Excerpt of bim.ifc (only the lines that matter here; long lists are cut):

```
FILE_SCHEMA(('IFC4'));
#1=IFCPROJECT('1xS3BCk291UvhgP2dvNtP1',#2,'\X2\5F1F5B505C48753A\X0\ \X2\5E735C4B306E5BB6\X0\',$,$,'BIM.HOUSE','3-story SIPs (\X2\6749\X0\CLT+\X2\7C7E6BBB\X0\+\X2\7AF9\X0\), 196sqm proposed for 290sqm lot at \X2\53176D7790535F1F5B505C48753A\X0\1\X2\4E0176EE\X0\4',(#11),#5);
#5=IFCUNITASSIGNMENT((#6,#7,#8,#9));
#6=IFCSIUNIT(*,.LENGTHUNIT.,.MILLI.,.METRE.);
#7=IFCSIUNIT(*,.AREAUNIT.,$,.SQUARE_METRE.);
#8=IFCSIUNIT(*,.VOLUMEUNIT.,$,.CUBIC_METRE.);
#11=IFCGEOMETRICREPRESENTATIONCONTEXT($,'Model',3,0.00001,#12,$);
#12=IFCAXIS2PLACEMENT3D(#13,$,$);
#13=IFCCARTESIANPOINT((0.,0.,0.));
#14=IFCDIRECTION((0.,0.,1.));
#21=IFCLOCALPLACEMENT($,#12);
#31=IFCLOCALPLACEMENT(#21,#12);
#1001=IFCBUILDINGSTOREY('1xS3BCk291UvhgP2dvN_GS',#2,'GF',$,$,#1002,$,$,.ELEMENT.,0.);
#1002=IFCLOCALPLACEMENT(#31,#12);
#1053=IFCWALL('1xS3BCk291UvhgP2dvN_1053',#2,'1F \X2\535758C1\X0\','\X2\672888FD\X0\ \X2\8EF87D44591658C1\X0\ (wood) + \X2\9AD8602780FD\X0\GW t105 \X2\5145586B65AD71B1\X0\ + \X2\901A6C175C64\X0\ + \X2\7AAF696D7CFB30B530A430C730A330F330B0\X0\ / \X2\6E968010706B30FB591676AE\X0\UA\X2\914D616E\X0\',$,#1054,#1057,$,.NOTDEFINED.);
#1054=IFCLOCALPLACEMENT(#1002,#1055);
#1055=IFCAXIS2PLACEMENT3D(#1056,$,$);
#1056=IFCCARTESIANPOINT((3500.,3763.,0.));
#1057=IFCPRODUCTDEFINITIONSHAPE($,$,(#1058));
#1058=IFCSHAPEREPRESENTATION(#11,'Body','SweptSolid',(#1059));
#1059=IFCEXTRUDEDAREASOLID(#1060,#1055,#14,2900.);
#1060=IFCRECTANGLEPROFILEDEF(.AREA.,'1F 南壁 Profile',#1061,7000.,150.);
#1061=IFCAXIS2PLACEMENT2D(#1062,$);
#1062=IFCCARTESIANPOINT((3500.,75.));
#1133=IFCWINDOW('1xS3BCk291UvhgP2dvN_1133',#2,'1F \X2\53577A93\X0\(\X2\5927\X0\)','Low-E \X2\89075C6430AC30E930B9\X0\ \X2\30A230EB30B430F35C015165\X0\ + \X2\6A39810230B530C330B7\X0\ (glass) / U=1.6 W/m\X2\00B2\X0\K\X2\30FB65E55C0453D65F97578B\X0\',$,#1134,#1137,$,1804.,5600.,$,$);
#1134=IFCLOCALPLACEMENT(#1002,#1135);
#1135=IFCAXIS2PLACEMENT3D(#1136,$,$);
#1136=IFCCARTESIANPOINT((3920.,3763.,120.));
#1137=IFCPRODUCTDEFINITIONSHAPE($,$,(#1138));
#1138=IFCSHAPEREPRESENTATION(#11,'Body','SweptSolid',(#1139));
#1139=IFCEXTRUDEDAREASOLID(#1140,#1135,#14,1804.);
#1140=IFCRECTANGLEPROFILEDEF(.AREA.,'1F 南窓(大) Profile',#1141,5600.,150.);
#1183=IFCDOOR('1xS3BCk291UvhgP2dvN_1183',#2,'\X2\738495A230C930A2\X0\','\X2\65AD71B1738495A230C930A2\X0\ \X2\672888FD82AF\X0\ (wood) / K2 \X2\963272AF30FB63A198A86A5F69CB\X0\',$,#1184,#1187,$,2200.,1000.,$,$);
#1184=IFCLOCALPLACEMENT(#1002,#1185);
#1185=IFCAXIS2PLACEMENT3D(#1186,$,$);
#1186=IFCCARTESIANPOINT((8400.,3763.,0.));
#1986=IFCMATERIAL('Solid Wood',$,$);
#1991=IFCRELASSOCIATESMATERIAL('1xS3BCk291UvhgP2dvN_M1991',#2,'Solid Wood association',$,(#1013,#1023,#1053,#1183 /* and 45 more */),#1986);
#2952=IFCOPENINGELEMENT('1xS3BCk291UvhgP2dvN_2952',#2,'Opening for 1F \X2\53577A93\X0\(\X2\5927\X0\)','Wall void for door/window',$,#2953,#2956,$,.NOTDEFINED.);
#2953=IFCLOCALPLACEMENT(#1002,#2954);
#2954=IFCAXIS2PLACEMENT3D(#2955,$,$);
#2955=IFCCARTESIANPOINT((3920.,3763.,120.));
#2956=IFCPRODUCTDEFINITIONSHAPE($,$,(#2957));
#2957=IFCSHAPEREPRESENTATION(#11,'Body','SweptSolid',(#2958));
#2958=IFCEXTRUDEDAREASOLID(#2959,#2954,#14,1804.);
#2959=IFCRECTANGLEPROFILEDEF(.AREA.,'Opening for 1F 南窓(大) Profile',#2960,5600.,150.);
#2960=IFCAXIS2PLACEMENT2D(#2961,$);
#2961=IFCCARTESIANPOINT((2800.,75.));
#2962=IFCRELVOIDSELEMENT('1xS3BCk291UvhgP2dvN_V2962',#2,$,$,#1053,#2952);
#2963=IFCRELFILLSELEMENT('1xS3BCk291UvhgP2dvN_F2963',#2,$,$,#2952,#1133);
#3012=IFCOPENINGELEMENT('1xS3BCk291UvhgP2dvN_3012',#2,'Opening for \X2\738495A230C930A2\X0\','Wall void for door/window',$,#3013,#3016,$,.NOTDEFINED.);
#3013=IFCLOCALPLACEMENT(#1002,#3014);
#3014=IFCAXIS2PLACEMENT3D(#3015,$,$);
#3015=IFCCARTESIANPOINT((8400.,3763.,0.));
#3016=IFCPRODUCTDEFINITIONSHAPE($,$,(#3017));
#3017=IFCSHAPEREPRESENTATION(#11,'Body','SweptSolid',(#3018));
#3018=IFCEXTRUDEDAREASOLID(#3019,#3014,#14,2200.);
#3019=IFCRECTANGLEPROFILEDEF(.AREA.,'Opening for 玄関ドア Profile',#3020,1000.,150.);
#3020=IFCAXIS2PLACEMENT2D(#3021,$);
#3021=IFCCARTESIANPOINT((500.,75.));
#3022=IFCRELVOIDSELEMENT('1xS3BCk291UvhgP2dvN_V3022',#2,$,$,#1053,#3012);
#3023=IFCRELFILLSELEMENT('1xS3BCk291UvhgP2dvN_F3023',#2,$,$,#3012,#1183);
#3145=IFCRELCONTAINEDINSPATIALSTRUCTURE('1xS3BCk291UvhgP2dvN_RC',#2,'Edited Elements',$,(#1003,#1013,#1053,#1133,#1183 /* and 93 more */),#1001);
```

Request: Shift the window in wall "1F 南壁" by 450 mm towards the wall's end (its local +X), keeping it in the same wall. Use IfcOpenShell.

```python
import ifcopenshell
import ifcopenshell.api.geometry
import ifcopenshell.util.placement

model = ifcopenshell.open("bim.ifc")

window = model.by_id(1133)
opening = window.FillsVoids[0].RelatingOpeningElement
wall = opening.VoidsElements[0].RelatingBuildingElement

wall_matrix = ifcopenshell.util.placement.get_local_placement(wall.ObjectPlacement)
shift = wall_matrix[:3, 0] * 450.0
before = ifcopenshell.util.placement.get_local_placement(window.ObjectPlacement)[:3, 3].copy()

# The window is not placed relative to its opening, so move both.
for product in (opening, window):
    matrix = ifcopenshell.util.placement.get_local_placement(product.ObjectPlacement)
    matrix[:3, 3] += shift
    ifcopenshell.api.geometry.edit_object_placement(model, product=product, matrix=matrix, is_si=False)

after = ifcopenshell.util.placement.get_local_placement(window.ObjectPlacement)[:3, 3]
print("window moved by", (after - before).round(3) + 0.0)

model.write("bim_v2.ifc")
```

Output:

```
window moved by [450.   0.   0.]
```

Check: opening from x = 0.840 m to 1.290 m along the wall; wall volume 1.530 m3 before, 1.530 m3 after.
